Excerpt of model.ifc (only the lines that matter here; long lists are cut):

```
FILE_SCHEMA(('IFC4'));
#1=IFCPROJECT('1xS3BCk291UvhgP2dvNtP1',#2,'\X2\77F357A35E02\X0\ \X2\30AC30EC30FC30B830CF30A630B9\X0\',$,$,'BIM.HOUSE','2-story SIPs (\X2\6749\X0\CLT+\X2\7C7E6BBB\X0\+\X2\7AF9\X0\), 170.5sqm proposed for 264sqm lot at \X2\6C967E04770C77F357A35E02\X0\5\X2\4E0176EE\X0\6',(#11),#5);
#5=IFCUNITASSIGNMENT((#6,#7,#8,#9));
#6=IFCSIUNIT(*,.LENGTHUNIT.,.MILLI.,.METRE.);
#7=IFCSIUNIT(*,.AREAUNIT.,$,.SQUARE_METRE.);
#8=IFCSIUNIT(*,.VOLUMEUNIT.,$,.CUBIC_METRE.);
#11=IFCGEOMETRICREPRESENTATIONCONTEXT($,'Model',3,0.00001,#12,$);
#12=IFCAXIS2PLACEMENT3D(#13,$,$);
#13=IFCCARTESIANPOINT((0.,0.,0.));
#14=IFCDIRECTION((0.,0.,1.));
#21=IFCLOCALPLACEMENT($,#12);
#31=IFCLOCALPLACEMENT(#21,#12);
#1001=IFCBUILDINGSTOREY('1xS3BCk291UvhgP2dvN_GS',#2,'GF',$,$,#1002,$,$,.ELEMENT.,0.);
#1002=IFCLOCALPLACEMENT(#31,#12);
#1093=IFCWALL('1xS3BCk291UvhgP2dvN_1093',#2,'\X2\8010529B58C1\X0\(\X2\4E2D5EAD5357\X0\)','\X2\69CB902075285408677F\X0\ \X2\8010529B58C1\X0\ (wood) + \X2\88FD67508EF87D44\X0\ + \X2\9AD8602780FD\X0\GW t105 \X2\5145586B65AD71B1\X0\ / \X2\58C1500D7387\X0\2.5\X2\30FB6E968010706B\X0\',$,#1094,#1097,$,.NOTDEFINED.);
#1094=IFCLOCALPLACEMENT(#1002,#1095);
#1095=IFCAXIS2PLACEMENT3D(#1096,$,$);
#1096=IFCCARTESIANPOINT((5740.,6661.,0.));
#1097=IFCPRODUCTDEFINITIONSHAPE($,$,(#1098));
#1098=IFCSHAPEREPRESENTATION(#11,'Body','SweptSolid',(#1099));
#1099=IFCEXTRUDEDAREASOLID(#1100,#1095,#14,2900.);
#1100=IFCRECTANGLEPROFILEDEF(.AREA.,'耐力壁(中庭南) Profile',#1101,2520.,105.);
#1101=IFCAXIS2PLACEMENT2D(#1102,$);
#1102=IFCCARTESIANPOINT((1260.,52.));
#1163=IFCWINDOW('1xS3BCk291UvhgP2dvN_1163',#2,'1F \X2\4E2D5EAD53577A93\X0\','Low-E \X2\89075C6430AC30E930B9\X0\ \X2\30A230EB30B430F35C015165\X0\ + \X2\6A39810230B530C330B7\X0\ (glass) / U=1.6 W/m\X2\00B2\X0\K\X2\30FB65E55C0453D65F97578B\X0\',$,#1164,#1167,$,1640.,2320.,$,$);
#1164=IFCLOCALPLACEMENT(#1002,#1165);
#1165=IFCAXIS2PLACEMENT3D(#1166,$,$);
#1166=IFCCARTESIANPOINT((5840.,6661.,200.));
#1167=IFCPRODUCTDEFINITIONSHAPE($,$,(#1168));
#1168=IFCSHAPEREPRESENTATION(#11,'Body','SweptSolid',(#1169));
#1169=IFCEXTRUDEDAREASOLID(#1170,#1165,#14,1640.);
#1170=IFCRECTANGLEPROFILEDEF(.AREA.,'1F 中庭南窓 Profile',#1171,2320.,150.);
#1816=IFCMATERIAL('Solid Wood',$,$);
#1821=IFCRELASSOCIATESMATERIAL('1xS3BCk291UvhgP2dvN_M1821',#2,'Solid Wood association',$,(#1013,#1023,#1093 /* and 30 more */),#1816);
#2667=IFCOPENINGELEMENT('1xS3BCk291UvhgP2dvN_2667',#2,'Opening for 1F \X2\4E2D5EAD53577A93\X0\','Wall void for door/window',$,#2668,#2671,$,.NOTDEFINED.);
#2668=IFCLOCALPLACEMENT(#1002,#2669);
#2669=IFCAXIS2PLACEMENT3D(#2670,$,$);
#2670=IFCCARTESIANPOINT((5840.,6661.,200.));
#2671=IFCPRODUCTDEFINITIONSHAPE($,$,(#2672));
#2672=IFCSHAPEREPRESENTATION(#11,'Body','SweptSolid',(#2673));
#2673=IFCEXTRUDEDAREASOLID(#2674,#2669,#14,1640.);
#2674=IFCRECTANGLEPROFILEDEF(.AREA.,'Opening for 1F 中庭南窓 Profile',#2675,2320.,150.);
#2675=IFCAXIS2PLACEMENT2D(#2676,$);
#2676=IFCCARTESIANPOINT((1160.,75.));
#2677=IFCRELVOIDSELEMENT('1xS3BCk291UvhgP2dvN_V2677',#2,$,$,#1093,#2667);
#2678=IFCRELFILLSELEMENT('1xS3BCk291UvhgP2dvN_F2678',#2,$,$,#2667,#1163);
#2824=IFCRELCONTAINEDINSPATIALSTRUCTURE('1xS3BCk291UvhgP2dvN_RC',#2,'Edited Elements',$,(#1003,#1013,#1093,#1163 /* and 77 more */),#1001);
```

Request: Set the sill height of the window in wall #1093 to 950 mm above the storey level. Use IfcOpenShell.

```python
import numpy as np
import ifcopenshell
import ifcopenshell.api.geometry
import ifcopenshell.geom
import ifcopenshell.util.element
import ifcopenshell.util.placement
import ifcopenshell.util.shape
import ifcopenshell.util.unit

model = ifcopenshell.open("model.ifc")
unit_scale = ifcopenshell.util.unit.calculate_unit_scale(model)

window = model.by_guid("1xS3BCk291UvhgP2dvN_1163")
opening = window.FillsVoids[0].RelatingOpeningElement
storey = ifcopenshell.util.element.get_container(window, ifc_class="IfcBuildingStorey")
level = ifcopenshell.util.placement.get_local_placement(storey.ObjectPlacement)[2, 3]

# The opening's origin need not be at the sill, so measure its lowest point.
shape = ifcopenshell.geom.create_shape(ifcopenshell.geom.settings(), opening)
bottom = ifcopenshell.util.shape.get_shape_bottom_elevation(shape, shape.geometry) / unit_scale
dz = level + 950.0 - bottom

shift = np.array([0.0, 0.0, dz])
# The window is not placed relative to its opening, so move both.
for product in (opening, window):
    matrix = ifcopenshell.util.placement.get_local_placement(product.ObjectPlacement)
    matrix[:3, 3] += shift
    ifcopenshell.api.geometry.edit_object_placement(model, product=product, matrix=matrix, is_si=False)

print(f"moved by {dz * unit_scale:+.3f} m")

model.write("model-out.ifc")
```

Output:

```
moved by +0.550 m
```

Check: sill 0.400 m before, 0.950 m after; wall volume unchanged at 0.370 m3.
